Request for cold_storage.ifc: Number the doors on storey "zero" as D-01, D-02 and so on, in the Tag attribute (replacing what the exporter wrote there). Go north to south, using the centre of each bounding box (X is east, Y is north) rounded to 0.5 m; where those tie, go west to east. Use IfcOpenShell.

First a look at what the model holds.

```python
import ifcopenshell
import ifcopenshell.util.element
import ifcopenshell.util.placement

model = ifcopenshell.open("cold_storage.ifc")
print(model.schema)
storey = next(s for s in model.by_type("IfcBuildingStorey") if s.Name == "zero")
doors = [e for e in ifcopenshell.util.element.get_decomposition(storey) if e.is_a("IfcDoor")]
for e in sorted(doors, key=lambda e: e.id()):
    origin = ifcopenshell.util.placement.get_local_placement(e.ObjectPlacement)[:3, 3]
    print(e.id(), e.Tag, e.Name, origin.round(2) + 0.0, sep=" | ")
```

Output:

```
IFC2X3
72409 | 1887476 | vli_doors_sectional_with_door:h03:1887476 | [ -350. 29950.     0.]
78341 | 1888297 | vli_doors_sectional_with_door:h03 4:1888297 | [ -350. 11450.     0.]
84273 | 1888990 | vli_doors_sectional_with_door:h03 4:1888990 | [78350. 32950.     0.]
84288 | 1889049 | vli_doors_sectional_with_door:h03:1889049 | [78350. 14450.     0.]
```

```python
import ifcopenshell
import ifcopenshell.geom
import ifcopenshell.util.element
import ifcopenshell.util.shape

model = ifcopenshell.open("cold_storage.ifc")
settings = ifcopenshell.geom.settings()
settings.set("use-world-coords", True)


def centre(element):
    shape = ifcopenshell.geom.create_shape(settings, element)
    return ifcopenshell.util.shape.get_bbox_centroid(shape.geometry)


storey = next(s for s in model.by_type("IfcBuildingStorey") if s.Name == "zero")
doors = [e for e in ifcopenshell.util.element.get_decomposition(storey) if e.is_a("IfcDoor")]

# Insertion points can sit at a corner or the storey origin, so sort by the geometry (in metres).
centres = {e: centre(e) for e in doors}
doors.sort(key=lambda e: (-round(centres[e][1] / 0.5), centres[e][0]))

for i, e in enumerate(doors, start=1):
    number = f"D-{i:02d}"
    e.Tag = number
    print(e.id(), number)

model.write("cold_storage_edited.ifc")
```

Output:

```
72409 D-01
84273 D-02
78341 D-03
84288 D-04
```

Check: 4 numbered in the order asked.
